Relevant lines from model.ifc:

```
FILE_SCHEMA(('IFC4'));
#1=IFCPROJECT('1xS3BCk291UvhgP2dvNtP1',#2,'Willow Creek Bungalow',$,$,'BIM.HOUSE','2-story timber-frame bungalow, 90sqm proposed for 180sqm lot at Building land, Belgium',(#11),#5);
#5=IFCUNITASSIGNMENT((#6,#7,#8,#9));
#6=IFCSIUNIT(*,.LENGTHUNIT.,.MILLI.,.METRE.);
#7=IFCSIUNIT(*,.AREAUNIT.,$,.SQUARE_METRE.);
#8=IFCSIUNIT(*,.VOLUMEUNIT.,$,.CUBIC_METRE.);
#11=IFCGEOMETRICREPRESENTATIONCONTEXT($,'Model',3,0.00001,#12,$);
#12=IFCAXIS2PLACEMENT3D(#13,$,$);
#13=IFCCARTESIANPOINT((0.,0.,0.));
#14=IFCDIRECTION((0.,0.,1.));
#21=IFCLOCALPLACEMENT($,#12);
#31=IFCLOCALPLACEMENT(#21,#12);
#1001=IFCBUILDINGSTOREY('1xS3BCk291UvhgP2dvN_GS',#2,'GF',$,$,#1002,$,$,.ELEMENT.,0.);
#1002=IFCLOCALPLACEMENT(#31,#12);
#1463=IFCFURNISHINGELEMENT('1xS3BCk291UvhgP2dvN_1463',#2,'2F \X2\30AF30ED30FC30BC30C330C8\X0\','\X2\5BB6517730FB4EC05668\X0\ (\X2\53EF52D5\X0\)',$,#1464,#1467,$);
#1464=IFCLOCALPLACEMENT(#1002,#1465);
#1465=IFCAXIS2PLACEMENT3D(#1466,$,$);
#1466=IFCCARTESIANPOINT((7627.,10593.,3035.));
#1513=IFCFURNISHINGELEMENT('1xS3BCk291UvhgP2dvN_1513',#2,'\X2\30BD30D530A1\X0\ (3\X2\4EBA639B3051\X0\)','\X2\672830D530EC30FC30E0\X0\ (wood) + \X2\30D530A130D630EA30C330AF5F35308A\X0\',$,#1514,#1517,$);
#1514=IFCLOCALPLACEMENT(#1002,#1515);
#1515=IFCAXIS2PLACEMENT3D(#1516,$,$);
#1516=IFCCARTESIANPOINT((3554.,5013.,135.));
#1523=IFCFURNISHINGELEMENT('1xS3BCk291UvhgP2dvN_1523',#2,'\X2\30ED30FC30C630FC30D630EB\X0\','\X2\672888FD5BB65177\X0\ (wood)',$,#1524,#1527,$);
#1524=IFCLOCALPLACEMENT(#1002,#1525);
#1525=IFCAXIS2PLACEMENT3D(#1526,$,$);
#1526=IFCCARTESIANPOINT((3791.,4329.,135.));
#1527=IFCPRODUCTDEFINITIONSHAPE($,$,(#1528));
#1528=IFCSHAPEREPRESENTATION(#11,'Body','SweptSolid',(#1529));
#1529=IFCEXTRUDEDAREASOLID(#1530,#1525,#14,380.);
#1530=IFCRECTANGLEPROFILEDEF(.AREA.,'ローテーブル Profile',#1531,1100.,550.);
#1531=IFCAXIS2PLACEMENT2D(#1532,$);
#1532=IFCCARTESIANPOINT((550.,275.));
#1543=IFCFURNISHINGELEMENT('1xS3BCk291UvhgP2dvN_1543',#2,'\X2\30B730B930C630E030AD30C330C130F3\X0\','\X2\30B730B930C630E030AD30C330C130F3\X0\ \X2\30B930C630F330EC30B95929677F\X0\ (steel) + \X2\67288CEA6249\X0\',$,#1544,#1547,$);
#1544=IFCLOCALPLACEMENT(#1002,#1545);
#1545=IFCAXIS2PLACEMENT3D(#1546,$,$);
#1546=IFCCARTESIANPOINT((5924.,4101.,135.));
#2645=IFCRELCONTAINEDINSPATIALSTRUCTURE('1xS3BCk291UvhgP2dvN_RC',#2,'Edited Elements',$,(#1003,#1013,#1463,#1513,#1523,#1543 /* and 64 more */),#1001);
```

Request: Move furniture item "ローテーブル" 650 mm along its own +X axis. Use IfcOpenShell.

```python
import ifcopenshell
import ifcopenshell.api.geometry
import ifcopenshell.util.placement
import ifcopenshell.util.unit

model = ifcopenshell.open("model.ifc")
unit_scale = ifcopenshell.util.unit.calculate_unit_scale(model)

item = model.by_guid("1xS3BCk291UvhgP2dvN_1523")
matrix = ifcopenshell.util.placement.get_local_placement(item.ObjectPlacement)
matrix[:3, 3] += matrix[:3, 0] * 0.65 / unit_scale
ifcopenshell.api.geometry.edit_object_placement(model, product=item, matrix=matrix, is_si=False)

print(ifcopenshell.util.placement.get_local_placement(item.ObjectPlacement).round(3) + 0.0)

model.write("model_updated.ifc")
```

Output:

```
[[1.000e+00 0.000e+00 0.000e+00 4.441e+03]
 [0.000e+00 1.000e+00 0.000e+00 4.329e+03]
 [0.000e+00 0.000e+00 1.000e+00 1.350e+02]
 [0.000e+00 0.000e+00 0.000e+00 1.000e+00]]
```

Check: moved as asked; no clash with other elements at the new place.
